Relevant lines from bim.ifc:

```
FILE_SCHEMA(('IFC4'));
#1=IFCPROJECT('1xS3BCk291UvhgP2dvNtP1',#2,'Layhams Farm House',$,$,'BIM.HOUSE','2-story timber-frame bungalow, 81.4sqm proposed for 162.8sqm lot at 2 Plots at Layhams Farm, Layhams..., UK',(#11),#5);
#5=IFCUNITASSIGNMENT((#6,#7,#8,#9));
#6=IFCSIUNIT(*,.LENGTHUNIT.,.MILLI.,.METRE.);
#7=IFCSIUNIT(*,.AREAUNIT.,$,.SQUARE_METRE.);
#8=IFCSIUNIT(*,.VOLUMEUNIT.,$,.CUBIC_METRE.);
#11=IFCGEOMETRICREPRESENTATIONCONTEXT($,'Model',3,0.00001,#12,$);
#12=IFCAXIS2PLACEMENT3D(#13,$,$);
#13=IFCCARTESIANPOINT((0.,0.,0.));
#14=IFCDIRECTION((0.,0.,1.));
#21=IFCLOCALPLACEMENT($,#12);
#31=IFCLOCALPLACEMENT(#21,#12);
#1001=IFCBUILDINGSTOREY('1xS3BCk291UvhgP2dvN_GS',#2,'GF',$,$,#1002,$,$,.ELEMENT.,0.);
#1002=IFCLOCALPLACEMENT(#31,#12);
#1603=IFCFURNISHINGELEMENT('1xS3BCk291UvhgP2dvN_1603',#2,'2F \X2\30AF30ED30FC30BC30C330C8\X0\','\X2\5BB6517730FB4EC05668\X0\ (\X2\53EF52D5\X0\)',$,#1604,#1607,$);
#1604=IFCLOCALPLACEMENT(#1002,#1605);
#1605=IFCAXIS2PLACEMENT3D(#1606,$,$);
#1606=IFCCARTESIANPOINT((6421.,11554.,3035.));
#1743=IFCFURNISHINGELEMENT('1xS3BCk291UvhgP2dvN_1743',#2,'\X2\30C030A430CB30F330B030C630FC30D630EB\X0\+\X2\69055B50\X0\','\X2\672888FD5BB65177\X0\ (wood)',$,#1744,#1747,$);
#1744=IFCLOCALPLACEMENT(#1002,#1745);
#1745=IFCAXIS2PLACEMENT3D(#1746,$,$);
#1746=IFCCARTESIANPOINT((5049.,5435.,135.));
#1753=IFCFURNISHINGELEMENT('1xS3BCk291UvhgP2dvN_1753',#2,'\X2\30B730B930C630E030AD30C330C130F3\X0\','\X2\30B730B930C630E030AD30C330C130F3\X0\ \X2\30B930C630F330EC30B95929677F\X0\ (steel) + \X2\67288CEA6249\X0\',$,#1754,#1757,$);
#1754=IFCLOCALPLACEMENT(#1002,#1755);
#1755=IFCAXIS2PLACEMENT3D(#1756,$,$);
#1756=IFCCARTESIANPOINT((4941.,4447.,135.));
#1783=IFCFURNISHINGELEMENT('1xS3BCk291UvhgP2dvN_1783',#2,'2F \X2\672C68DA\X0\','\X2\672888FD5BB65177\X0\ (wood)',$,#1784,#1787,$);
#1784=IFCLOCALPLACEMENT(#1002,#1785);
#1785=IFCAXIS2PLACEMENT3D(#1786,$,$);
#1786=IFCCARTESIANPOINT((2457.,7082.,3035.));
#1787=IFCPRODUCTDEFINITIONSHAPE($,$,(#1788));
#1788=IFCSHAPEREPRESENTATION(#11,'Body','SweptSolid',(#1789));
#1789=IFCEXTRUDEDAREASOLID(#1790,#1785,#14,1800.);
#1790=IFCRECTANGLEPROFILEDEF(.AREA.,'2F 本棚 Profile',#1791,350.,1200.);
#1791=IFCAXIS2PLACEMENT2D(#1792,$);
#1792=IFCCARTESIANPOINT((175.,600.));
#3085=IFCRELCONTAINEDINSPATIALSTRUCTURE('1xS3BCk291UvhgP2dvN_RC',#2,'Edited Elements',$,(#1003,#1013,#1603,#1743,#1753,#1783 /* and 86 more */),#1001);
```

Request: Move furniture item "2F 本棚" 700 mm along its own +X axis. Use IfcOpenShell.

```python
import ifcopenshell
import ifcopenshell.api.geometry
import ifcopenshell.util.placement
import ifcopenshell.util.unit

model = ifcopenshell.open("bim.ifc")
unit_scale = ifcopenshell.util.unit.calculate_unit_scale(model)

item = model.by_guid("1xS3BCk291UvhgP2dvN_1783")
matrix = ifcopenshell.util.placement.get_local_placement(item.ObjectPlacement)
matrix[:3, 3] += matrix[:3, 0] * 0.7 / unit_scale
ifcopenshell.api.geometry.edit_object_placement(model, product=item, matrix=matrix, is_si=False)

print(ifcopenshell.util.placement.get_local_placement(item.ObjectPlacement).round(3) + 0.0)

model.write("bim_rev.ifc")
```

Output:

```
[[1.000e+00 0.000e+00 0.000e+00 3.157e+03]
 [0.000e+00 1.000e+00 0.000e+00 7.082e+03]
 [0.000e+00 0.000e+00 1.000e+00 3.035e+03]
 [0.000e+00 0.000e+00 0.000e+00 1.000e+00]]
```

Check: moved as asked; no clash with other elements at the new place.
